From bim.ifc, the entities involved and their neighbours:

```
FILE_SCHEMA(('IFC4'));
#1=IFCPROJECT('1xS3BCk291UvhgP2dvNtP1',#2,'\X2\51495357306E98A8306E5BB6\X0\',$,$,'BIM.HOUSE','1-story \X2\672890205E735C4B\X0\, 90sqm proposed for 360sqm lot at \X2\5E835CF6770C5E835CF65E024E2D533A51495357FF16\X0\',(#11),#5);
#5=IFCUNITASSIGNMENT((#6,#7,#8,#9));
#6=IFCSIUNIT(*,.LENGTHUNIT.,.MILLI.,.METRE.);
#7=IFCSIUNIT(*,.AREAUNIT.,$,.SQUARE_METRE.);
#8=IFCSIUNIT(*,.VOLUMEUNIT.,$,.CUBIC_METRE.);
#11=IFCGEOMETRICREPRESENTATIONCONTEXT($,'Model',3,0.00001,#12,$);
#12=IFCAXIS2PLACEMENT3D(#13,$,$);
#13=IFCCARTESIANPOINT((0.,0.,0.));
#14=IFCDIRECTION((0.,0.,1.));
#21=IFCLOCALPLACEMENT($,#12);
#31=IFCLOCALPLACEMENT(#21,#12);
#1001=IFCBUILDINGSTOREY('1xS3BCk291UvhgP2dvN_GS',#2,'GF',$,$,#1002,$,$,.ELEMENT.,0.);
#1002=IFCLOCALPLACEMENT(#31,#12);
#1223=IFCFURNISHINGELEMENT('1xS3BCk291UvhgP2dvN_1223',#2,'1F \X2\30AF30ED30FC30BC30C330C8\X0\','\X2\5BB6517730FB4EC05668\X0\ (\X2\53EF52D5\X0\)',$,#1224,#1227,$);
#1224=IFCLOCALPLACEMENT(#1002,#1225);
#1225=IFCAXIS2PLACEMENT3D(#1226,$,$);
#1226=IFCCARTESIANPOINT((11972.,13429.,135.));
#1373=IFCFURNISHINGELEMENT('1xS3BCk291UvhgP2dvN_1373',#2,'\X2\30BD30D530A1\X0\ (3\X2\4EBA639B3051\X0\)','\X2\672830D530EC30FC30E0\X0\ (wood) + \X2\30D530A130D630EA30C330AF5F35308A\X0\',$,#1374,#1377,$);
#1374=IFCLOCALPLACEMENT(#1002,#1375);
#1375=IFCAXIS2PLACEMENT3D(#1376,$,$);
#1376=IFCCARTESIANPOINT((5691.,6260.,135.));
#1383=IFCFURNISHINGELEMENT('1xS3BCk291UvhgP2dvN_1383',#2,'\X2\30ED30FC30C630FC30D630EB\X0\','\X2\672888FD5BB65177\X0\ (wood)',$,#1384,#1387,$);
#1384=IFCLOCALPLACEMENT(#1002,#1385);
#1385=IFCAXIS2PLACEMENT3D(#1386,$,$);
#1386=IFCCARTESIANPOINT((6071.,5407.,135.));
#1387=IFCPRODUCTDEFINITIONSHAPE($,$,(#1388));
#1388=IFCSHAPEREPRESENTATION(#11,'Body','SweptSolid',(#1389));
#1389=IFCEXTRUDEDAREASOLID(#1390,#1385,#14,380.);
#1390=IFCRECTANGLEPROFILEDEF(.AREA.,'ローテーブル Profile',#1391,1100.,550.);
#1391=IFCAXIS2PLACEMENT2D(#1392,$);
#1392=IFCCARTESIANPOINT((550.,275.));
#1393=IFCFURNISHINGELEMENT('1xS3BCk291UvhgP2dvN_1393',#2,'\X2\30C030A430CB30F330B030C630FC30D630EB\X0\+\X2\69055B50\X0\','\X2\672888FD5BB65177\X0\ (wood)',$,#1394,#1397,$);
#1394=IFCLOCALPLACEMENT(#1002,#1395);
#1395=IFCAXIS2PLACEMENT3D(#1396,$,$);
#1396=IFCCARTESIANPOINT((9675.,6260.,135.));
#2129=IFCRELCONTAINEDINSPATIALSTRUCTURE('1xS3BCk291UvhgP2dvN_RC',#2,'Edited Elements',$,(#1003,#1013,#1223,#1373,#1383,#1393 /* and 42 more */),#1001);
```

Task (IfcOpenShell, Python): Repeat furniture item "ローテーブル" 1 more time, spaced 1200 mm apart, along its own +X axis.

```python
import ifcopenshell
import ifcopenshell.api.geometry
import ifcopenshell.api.root
import ifcopenshell.util.element
import ifcopenshell.util.placement
import ifcopenshell.util.unit

model = ifcopenshell.open("bim.ifc")
unit_scale = ifcopenshell.util.unit.calculate_unit_scale(model)


def reuse_history(source, copy):
    """copy_class also copies each property set's owner history, people and application; keep the originals."""
    for rel in copy.IsDefinedBy:
        if rel.is_a("IfcRelDefinesByProperties") and (history := rel.RelatingPropertyDefinition.OwnerHistory):
            rel.RelatingPropertyDefinition.OwnerHistory = source.OwnerHistory
            ifcopenshell.util.element.remove_deep2(model, history)


source = model.by_guid("1xS3BCk291UvhgP2dvN_1383")
base = ifcopenshell.util.placement.get_local_placement(source.ObjectPlacement)
step = base[:3, 0] * 1.2 / unit_scale

for i in range(1, 2):
    copy = ifcopenshell.api.root.copy_class(model, product=source)
    copy.Representation = ifcopenshell.util.element.copy_deep(
        model, source.Representation, exclude=["IfcGeometricRepresentationContext", "IfcRepresentationMap"]
    )
    reuse_history(source, copy)
    matrix = base.copy()
    matrix[:3, 3] += i * step
    print("added at", matrix[:3, 3].round(3) + 0.0)
    ifcopenshell.api.geometry.edit_object_placement(model, product=copy, matrix=matrix, is_si=False)

model.write("bim_edited.ifc")
```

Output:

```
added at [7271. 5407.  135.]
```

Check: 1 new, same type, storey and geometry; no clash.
